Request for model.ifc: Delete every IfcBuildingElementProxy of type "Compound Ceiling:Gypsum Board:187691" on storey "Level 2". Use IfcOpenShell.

First a look at what the model holds.

```python
import ifcopenshell
import ifcopenshell.util.element

model = ifcopenshell.open("model.ifc")
print(model.schema)
storey = next(s for s in model.by_type("IfcBuildingStorey") if s.Name == "Level 2")
proxies = [e for e in ifcopenshell.util.element.get_decomposition(storey) if e.is_a("IfcBuildingElementProxy")]
seen = {}
for e in proxies:
    element_type = ifcopenshell.util.element.get_type(e)
    name = element_type.Name if element_type not in (None, e) else None
    seen[name] = seen.get(name, 0) + 1
for name, count in sorted(seen.items(), key=str):
    print(count, "x", name)
```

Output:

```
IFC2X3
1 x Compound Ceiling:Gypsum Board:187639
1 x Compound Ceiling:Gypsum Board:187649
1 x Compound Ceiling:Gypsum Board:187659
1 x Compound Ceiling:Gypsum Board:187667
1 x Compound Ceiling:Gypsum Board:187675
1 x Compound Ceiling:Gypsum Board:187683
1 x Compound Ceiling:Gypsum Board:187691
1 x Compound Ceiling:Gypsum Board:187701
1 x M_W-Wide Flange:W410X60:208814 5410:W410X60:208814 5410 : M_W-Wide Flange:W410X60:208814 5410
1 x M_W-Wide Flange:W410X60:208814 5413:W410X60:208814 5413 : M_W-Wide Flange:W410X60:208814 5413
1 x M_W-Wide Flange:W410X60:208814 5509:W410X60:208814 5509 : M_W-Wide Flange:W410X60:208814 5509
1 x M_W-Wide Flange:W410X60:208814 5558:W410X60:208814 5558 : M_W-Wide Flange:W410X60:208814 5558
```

```python
import ifcopenshell
import ifcopenshell.api.root
import ifcopenshell.util.element

model = ifcopenshell.open("model.ifc")

storey = next(s for s in model.by_type("IfcBuildingStorey") if s.Name == "Level 2")
proxies = [e for e in ifcopenshell.util.element.get_decomposition(storey) if e.is_a("IfcBuildingElementProxy")]
targets = [e for e in proxies if (t := ifcopenshell.util.element.get_type(e)) not in (None, e) and t.Name == "Compound Ceiling:Gypsum Board:187691"]

for e in targets:
    ifcopenshell.api.root.remove_product(model, product=e)
print(len(targets), "removed")

model.write("model_rev.ifc")
```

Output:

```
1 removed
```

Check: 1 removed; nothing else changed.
